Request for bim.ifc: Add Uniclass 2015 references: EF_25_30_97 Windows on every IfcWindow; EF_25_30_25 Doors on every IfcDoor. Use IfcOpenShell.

First a look at what the model holds.

```python
import ifcopenshell

model = ifcopenshell.open("bim.ifc")
print(model.schema)
print("classifications:", [c.Name for c in model.by_type("IfcClassification")])
for ifc_class in ("IfcDoor", "IfcRoof", "IfcStair", "IfcWall", "IfcWindow"):
    print(ifc_class, len(model.by_type(ifc_class)))
```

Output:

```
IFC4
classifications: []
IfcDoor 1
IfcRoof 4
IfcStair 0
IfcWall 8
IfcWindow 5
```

```python
import ifcopenshell
import ifcopenshell.api.classification

model = ifcopenshell.open("bim.ifc")

system = ifcopenshell.api.classification.add_classification(model, classification="Uniclass 2015")

codes = {
    "IfcWindow": ("EF_25_30_97", "Windows"),
    "IfcDoor": ("EF_25_30_25", "Doors"),
}
for ifc_class, (code, name) in codes.items():
    products = model.by_type(ifc_class)
    ifcopenshell.api.classification.add_reference(
        model, products=products, classification=system, identification=code, name=name
    )
    print(code, len(products))

model.write("bim_edited.ifc")
```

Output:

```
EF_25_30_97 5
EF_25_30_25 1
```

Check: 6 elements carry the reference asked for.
